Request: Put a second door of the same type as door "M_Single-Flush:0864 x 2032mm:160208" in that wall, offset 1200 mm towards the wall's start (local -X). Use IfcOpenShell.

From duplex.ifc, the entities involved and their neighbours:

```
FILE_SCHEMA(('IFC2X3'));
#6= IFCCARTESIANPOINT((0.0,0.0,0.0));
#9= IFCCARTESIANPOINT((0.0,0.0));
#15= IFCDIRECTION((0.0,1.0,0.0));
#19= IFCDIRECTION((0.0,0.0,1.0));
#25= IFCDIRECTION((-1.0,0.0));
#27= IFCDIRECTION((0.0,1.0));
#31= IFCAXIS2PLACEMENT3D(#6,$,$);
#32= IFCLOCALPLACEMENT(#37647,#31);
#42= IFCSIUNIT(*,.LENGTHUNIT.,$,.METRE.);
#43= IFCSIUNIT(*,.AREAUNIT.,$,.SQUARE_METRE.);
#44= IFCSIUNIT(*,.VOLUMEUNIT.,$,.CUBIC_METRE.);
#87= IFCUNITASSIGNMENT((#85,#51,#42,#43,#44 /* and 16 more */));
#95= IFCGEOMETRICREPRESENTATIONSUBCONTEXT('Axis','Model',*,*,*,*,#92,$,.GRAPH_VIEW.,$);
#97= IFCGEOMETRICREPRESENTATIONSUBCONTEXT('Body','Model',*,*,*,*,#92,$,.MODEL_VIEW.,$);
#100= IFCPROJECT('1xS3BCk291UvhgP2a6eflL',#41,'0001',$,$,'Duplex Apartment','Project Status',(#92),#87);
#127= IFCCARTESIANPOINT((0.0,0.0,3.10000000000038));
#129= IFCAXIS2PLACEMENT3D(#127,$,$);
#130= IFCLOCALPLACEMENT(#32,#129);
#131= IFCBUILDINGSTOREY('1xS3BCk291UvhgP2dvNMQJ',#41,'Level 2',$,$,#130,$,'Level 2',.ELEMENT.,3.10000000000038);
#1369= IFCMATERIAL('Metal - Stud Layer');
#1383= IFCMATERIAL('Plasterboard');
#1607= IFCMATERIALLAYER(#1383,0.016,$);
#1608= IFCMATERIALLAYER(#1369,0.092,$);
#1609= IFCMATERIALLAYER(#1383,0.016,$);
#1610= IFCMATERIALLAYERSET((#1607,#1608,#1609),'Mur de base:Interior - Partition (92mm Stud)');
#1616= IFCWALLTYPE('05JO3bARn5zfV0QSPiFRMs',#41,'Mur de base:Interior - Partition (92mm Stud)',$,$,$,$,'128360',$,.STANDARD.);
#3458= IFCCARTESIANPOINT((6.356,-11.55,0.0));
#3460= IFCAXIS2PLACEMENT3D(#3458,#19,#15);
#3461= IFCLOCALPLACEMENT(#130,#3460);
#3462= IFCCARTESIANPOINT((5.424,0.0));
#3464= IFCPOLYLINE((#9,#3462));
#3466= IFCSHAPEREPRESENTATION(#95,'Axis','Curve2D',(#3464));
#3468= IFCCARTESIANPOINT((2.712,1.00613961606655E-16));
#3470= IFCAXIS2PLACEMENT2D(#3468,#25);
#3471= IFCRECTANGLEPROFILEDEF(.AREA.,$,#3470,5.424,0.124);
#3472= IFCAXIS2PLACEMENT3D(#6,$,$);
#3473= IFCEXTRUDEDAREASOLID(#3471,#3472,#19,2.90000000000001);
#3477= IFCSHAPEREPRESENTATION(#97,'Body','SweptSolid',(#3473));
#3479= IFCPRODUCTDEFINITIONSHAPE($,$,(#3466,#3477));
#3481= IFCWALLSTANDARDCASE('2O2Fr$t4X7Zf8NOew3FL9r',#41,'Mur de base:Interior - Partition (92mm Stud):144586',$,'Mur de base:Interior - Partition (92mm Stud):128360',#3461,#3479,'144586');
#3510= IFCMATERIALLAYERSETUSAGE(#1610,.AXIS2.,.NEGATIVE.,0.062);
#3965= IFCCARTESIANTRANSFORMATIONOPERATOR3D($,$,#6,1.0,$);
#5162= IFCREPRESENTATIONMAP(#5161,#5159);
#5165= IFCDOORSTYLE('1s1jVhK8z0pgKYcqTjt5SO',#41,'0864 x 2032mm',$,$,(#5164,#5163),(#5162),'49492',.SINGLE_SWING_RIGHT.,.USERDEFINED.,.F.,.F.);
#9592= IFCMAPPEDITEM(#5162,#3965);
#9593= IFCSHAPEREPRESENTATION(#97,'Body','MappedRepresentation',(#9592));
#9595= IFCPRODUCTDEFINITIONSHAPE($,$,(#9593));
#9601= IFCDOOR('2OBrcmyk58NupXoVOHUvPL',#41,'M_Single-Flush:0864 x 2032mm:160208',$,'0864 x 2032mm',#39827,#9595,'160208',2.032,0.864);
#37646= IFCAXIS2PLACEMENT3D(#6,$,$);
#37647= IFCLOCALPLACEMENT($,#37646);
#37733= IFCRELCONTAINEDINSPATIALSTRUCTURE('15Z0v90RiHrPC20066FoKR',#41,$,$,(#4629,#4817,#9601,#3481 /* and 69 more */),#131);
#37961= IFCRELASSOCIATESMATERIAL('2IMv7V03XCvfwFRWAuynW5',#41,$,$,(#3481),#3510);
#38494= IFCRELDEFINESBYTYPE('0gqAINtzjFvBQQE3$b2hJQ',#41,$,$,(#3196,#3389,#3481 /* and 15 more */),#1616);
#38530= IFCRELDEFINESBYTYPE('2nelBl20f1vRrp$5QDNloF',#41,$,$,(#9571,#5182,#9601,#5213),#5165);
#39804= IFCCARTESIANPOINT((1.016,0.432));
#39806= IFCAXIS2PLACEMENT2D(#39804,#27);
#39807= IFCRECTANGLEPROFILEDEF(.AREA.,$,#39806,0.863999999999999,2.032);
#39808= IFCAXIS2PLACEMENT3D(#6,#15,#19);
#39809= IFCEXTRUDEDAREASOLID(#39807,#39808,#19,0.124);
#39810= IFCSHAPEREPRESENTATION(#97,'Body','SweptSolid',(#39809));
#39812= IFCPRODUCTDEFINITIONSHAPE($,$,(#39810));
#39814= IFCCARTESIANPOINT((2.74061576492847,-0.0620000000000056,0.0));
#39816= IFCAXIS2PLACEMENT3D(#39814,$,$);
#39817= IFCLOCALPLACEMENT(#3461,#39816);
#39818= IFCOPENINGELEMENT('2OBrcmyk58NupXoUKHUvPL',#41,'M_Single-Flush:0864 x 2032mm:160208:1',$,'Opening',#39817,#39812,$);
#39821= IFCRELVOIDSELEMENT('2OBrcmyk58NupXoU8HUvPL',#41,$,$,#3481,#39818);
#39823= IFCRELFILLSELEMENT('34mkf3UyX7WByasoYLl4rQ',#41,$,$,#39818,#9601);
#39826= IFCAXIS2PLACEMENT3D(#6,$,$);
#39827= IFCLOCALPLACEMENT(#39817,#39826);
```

```python
import ifcopenshell
import ifcopenshell.api.feature
import ifcopenshell.api.geometry
import ifcopenshell.api.root
import ifcopenshell.geom
import ifcopenshell.util.element
import ifcopenshell.util.placement
import ifcopenshell.util.shape

model = ifcopenshell.open("duplex.ifc")
settings = ifcopenshell.geom.settings()


def volume(element):
    """Net volume in cubic metres, openings subtracted."""
    shape = ifcopenshell.geom.create_shape(settings, element)
    return ifcopenshell.util.shape.get_volume(shape.geometry)


def reuse_history(source, copy):
    """copy_class also copies each property set's owner history, people and application; keep the originals."""
    for rel in copy.IsDefinedBy:
        if rel.is_a("IfcRelDefinesByProperties") and (history := rel.RelatingPropertyDefinition.OwnerHistory):
            rel.RelatingPropertyDefinition.OwnerHistory = source.OwnerHistory
            ifcopenshell.util.element.remove_deep2(model, history)


door = model.by_guid("2OBrcmyk58NupXoVOHUvPL")
opening = door.FillsVoids[0].RelatingOpeningElement
wall = opening.VoidsElements[0].RelatingBuildingElement
before = volume(wall)
shift = ifcopenshell.util.placement.get_local_placement(wall.ObjectPlacement)[:3, 0] * -1.2

# copy_class copies the void relationship, type, container and properties, but no geometry.
new_opening = ifcopenshell.api.root.copy_class(model, product=opening)
new_opening.Representation = ifcopenshell.util.element.copy_deep(
    model, opening.Representation, exclude=["IfcGeometricRepresentationContext", "IfcRepresentationMap"]
)
new_opening.Name = "M_Single-Flush:0864 x 2032mm"
new_door = ifcopenshell.api.root.copy_class(model, product=door)
new_door.Representation = ifcopenshell.util.element.copy_deep(
    model, door.Representation, exclude=["IfcGeometricRepresentationContext", "IfcRepresentationMap"]
)
new_door.Name = "M_Single-Flush:0864 x 2032mm"
new_door.Tag = None
reuse_history(door, new_door)
fills = ifcopenshell.api.feature.add_filling(model, opening=new_opening, element=new_door)
fills.OwnerHistory = new_door.OwnerHistory  # required in IFC2X3

for old, new in ((opening, new_opening), (door, new_door)):
    matrix = ifcopenshell.util.placement.get_local_placement(old.ObjectPlacement)
    matrix[:3, 3] += shift
    ifcopenshell.api.geometry.edit_object_placement(model, product=new, matrix=matrix, is_si=False)

after = volume(wall)

print(f"wall volume {before:.3f} -> {after:.3f} m3")

model.write("duplex_v2.ifc")
```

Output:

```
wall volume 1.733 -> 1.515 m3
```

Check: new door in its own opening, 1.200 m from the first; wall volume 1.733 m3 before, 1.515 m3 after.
